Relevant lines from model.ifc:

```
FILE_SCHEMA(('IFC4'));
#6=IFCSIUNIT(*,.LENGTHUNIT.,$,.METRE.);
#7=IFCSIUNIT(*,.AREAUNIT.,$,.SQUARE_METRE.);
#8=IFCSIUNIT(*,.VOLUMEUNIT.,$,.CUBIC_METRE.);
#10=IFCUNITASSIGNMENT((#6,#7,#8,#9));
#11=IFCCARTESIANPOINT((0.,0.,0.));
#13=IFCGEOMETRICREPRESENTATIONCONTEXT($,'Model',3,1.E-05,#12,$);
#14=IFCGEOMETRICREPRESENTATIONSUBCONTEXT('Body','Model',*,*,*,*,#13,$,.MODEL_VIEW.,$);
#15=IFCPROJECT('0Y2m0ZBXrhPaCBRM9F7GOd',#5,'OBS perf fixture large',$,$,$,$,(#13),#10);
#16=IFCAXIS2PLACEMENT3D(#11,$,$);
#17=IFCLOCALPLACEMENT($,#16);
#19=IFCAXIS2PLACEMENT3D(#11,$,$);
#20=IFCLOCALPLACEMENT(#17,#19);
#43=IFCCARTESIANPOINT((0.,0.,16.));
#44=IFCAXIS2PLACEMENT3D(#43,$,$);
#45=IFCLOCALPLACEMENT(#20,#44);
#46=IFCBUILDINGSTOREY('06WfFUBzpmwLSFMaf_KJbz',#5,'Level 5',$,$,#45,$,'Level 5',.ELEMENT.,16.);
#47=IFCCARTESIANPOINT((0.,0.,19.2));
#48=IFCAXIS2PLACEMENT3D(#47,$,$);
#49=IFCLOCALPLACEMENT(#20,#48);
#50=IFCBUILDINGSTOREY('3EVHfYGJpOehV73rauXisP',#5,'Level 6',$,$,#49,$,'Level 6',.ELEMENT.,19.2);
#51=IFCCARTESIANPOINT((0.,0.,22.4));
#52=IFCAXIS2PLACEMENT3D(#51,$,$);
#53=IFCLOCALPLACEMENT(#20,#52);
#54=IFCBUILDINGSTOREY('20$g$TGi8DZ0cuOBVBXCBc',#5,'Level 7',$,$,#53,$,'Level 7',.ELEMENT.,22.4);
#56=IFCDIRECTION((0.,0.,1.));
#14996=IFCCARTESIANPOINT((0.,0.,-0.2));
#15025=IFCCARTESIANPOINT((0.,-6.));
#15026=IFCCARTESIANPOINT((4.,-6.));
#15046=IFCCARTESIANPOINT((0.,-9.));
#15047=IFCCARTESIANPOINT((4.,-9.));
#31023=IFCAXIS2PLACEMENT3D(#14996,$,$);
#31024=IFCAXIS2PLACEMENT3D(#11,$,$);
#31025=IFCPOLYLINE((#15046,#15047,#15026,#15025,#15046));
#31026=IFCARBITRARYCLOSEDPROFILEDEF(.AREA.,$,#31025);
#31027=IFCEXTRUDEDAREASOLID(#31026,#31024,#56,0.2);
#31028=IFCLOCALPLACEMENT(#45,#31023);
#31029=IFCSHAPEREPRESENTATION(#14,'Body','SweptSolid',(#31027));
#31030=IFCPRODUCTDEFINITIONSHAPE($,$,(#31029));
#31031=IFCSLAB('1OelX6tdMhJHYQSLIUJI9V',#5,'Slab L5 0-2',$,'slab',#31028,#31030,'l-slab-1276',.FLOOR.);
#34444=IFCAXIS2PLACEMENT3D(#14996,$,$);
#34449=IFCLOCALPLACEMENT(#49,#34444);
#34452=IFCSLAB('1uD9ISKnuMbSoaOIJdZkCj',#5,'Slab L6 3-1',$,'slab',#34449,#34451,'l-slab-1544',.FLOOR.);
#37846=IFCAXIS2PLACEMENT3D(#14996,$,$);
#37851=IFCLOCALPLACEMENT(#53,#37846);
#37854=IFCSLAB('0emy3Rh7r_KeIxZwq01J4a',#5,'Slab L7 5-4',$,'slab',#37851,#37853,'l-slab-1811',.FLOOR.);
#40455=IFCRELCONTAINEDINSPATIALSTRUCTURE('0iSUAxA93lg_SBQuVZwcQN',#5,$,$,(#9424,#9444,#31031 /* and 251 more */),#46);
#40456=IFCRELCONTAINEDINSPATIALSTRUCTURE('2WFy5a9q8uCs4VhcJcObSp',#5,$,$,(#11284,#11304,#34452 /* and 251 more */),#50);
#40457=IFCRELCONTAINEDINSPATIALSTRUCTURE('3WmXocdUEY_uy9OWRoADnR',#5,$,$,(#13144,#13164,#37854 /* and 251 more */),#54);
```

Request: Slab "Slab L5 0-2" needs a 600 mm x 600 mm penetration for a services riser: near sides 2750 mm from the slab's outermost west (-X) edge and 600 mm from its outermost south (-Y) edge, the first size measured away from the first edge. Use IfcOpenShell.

```python
import numpy as np
import ifcopenshell
import ifcopenshell.api.feature
import ifcopenshell.api.geometry
import ifcopenshell.api.root
import ifcopenshell.geom
import ifcopenshell.util.placement
import ifcopenshell.util.representation
import ifcopenshell.util.shape
import ifcopenshell.util.unit

model = ifcopenshell.open("model.ifc")
unit_scale = ifcopenshell.util.unit.calculate_unit_scale(model)
settings = ifcopenshell.geom.settings()


def volume(element):
    """Net volume in cubic metres, openings subtracted."""
    shape = ifcopenshell.geom.create_shape(settings, element)
    return ifcopenshell.util.shape.get_volume(shape.geometry)


slab = model.by_guid("1OelX6tdMhJHYQSLIUJI9V")
before = volume(slab)

# Extent in the slab's own axes, in metres. The edges named are its -X and -Y sides.
slab_shape = ifcopenshell.geom.create_shape(settings, slab)
vertices = ifcopenshell.util.shape.get_vertices(slab_shape.geometry)
x_min, y_min, bottom = vertices.min(axis=0)
top = vertices[:, 2].max()

opening = ifcopenshell.api.root.create_entity(model, ifc_class="IfcOpeningElement", name="Services riser opening", predefined_type="OPENING")
context = ifcopenshell.util.representation.get_context(model, "Model", "Body", "MODEL_VIEW")
width, depth = 0.6, 0.6
outline = [(0.0, 0.0), (width, 0.0), (width, depth), (0.0, depth), (0.0, 0.0)]
# Overshoot both faces by 50 mm so the cut is clean.
shape = ifcopenshell.api.geometry.add_slab_representation(
    model, context=context, depth=top - bottom + 0.1, polyline=outline
)
ifcopenshell.api.geometry.assign_representation(model, product=opening, representation=shape)

matrix = ifcopenshell.util.placement.get_local_placement(slab.ObjectPlacement)
matrix[:, 3] = matrix @ np.append(np.array([x_min + 2.75, y_min + 0.6, bottom - 0.05]) / unit_scale, 1.0)
ifcopenshell.api.geometry.edit_object_placement(model, product=opening, matrix=matrix, is_si=False)
ifcopenshell.api.feature.add_feature(model, feature=opening, element=slab)

after = volume(slab)

print(f"slab volume {before:.3f} -> {after:.3f} m3")

model.write("model_updated.ifc")
```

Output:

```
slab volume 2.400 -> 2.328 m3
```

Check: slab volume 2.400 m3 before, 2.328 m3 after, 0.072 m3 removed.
